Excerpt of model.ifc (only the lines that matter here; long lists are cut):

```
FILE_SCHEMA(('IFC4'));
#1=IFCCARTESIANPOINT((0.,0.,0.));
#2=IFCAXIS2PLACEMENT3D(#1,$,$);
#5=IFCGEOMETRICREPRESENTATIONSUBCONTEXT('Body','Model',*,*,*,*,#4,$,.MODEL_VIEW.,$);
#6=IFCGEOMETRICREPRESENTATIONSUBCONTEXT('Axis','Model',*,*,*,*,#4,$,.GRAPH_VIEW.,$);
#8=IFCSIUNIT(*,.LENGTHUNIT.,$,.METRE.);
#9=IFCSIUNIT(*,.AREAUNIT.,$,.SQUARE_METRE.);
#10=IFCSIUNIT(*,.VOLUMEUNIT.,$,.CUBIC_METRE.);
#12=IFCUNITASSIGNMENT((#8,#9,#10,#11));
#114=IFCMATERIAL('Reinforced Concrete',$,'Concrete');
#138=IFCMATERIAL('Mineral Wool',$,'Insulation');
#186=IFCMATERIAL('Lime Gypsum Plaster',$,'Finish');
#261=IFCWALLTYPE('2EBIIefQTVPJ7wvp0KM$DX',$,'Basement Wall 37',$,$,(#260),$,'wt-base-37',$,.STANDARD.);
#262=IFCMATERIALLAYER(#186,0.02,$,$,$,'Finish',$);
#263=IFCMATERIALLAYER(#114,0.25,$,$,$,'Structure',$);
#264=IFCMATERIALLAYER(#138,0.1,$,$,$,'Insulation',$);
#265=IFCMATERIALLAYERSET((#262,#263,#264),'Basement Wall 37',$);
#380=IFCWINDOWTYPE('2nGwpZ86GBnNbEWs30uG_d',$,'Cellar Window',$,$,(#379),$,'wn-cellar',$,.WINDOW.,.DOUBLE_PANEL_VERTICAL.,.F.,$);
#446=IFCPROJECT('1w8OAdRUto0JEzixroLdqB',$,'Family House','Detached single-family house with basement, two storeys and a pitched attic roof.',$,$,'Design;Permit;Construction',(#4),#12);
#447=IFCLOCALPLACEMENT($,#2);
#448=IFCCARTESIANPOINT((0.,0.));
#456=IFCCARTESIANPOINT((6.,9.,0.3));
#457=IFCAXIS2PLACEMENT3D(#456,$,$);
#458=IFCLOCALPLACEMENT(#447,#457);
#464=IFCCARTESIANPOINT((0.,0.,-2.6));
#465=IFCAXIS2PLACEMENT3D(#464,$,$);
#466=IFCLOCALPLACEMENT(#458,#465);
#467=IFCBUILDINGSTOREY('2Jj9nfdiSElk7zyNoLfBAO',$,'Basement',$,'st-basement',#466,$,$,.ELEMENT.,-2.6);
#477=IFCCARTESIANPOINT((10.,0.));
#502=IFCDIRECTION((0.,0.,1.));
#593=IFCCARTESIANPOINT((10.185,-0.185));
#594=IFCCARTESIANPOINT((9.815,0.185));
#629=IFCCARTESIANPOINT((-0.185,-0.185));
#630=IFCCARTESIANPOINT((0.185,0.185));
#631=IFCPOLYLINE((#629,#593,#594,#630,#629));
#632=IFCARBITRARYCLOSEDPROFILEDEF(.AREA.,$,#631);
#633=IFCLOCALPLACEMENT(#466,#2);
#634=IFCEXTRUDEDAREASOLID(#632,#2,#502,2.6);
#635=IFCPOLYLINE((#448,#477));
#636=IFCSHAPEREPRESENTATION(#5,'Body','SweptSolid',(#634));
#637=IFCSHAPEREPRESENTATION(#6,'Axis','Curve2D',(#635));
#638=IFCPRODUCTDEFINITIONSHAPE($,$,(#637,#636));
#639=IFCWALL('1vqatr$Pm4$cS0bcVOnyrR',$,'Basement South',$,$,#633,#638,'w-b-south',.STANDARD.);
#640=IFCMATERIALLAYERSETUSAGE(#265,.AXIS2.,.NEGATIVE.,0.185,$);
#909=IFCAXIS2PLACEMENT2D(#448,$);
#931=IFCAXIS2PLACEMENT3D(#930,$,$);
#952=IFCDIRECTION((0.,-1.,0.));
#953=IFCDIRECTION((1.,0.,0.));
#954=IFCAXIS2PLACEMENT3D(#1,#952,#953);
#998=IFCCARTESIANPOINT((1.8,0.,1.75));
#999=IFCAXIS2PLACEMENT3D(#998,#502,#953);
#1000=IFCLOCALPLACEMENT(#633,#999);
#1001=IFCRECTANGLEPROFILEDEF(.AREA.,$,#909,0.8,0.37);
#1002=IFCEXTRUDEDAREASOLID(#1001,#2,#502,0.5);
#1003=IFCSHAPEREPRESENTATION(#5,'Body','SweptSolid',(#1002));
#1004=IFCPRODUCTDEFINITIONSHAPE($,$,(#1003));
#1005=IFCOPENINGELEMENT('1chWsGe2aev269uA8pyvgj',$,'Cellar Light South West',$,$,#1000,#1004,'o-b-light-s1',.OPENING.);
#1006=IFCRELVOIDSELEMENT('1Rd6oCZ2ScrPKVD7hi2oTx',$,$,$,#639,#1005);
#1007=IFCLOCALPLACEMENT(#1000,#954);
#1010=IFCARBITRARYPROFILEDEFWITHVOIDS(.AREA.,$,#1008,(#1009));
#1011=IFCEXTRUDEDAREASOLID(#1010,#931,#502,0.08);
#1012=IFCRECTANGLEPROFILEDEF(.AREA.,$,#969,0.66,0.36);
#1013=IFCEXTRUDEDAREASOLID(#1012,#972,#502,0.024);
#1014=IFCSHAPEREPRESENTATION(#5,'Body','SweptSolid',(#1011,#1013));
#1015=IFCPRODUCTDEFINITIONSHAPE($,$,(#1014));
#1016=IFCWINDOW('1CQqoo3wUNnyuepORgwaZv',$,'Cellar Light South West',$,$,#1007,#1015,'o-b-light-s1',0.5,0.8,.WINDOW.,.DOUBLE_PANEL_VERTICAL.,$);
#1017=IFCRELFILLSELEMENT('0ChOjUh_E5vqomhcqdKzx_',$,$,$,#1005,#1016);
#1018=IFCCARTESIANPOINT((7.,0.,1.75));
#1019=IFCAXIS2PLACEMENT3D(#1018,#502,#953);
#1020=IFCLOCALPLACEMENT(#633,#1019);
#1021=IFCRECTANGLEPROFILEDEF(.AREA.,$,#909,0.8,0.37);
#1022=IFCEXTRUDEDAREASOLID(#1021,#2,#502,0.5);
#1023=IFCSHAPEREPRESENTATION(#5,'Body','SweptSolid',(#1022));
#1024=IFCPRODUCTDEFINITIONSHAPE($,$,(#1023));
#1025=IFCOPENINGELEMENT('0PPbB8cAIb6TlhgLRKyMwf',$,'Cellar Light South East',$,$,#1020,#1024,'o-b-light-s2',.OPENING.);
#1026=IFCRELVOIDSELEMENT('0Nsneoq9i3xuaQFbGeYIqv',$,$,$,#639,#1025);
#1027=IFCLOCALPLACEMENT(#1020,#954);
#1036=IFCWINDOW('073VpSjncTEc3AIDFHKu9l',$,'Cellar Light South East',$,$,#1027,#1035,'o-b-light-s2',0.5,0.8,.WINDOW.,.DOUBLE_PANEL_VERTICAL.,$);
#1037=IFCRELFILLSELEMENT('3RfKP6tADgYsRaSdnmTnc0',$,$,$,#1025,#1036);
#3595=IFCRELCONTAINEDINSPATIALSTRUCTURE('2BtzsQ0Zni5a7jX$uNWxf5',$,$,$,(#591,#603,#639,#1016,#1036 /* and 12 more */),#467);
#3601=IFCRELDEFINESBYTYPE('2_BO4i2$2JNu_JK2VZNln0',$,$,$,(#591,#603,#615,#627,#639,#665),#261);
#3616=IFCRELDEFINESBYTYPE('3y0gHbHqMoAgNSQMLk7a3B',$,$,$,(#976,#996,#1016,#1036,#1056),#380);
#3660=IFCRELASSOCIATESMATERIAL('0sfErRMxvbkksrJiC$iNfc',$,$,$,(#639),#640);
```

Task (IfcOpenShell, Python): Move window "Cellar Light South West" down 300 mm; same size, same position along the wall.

```python
import numpy as np
import ifcopenshell
import ifcopenshell.api.geometry
import ifcopenshell.util.placement
import ifcopenshell.util.unit

model = ifcopenshell.open("model.ifc")
unit_scale = ifcopenshell.util.unit.calculate_unit_scale(model)

window = model.by_guid("1CQqoo3wUNnyuepORgwaZv")
opening = window.FillsVoids[0].RelatingOpeningElement
dz = -0.3

shift = np.array([0.0, 0.0, dz])
# The window is placed relative to its opening, so it follows when the opening moves.
matrix = ifcopenshell.util.placement.get_local_placement(opening.ObjectPlacement)
matrix[:3, 3] += shift
ifcopenshell.api.geometry.edit_object_placement(
    model, product=opening, matrix=matrix, is_si=False, should_transform_children=True
)

print(f"moved by {dz * unit_scale:+.3f} m")

model.write("model_updated.ifc")
```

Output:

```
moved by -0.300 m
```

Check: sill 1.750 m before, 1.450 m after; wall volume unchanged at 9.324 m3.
